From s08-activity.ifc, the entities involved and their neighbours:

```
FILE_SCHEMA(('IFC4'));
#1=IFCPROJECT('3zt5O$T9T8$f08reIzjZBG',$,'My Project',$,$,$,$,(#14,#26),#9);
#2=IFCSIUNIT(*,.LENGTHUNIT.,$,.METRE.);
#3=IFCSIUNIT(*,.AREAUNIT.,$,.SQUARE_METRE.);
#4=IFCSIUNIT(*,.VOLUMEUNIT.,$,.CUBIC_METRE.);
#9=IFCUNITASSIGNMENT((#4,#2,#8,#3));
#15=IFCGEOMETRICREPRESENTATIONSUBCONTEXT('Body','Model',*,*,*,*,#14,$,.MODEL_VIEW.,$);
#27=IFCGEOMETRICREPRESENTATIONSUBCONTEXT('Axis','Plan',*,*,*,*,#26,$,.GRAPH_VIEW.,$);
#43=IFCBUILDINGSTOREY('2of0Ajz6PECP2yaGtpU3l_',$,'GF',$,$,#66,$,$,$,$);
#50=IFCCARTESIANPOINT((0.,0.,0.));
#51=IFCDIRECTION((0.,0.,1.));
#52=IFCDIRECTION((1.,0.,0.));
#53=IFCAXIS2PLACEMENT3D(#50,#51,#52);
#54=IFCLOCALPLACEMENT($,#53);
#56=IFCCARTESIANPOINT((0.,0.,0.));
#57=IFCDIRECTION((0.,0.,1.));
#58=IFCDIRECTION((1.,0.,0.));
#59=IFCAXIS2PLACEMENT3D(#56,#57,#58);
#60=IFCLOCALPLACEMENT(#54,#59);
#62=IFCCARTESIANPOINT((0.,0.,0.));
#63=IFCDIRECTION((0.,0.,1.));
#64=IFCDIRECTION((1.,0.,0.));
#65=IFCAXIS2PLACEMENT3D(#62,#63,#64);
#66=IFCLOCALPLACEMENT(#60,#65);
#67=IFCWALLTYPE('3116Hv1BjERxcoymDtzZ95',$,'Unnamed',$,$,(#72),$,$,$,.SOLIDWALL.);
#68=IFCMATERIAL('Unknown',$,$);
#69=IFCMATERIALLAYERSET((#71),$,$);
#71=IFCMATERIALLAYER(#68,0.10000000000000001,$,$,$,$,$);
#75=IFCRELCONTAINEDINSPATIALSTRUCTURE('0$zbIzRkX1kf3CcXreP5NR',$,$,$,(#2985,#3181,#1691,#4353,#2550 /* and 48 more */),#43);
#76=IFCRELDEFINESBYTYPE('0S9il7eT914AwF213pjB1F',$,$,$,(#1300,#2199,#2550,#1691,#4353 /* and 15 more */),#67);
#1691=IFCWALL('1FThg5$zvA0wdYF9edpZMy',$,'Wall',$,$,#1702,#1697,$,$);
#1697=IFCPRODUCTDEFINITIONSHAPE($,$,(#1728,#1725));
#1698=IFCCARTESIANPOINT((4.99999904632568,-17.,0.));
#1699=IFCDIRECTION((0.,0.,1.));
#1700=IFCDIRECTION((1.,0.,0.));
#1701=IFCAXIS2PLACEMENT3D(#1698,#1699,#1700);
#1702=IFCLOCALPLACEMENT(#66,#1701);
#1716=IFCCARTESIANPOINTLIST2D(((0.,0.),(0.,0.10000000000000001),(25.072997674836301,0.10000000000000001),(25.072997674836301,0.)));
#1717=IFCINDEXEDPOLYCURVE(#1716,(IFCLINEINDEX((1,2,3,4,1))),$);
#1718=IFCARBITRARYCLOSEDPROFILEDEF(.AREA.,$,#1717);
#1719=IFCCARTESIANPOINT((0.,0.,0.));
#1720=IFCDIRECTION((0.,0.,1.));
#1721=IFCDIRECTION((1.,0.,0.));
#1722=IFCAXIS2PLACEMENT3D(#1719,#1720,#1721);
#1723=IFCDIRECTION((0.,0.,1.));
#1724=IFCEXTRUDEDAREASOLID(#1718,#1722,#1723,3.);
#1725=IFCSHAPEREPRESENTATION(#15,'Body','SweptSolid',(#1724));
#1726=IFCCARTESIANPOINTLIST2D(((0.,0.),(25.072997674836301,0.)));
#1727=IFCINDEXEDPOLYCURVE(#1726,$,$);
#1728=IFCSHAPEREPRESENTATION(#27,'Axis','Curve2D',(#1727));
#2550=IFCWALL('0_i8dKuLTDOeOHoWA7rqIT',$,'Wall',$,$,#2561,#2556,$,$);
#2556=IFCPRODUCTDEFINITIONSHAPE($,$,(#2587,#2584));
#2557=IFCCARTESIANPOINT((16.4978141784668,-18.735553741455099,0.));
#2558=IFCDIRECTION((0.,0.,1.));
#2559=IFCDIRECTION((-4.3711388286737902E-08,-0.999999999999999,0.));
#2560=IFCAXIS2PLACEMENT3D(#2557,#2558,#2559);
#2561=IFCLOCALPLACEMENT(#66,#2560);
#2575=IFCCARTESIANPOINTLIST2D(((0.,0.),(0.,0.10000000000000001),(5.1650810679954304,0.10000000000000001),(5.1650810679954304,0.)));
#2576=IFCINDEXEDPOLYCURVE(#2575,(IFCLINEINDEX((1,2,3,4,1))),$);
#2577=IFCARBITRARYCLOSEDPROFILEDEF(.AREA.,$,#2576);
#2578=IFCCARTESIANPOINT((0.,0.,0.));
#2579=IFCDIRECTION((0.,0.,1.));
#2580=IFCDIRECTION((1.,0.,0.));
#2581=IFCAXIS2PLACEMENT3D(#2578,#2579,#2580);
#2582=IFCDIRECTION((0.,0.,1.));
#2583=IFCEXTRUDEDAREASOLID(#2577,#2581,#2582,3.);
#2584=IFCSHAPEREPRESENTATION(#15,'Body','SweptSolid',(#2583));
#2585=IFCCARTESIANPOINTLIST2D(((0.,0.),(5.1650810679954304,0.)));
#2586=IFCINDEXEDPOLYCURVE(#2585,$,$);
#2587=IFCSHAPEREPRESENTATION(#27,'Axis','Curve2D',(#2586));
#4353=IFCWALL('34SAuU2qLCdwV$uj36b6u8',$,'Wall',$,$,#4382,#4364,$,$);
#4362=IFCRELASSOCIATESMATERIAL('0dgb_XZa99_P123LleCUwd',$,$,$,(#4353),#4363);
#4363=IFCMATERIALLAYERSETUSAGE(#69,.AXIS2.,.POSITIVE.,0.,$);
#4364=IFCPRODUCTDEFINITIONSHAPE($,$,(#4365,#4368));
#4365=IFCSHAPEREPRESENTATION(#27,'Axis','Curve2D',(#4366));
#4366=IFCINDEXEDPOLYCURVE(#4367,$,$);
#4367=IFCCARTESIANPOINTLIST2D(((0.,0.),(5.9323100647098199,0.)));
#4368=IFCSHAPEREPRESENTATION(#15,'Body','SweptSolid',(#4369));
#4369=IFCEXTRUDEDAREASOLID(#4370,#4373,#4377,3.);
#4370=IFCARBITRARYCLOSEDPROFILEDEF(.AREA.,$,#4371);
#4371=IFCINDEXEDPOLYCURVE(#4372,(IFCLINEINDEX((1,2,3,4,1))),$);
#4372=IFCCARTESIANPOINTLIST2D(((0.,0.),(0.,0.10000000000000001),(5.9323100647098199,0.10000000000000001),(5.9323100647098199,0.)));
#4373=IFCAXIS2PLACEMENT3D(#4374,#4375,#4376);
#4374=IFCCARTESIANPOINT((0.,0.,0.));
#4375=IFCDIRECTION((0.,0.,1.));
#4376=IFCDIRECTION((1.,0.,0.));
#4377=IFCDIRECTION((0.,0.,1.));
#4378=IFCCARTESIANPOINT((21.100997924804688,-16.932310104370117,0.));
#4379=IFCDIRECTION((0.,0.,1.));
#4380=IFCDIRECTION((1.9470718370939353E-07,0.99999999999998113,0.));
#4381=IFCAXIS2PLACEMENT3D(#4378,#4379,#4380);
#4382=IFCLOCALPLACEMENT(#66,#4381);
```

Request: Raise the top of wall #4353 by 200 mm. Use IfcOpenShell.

```python
import ifcopenshell
import ifcopenshell.geom
import ifcopenshell.util.representation
import ifcopenshell.util.shape
import ifcopenshell.util.unit

model = ifcopenshell.open("s08-activity.ifc")
unit_scale = ifcopenshell.util.unit.calculate_unit_scale(model)
settings = ifcopenshell.geom.settings()


def volume(element):
    """Net volume in cubic metres, openings subtracted."""
    shape = ifcopenshell.geom.create_shape(settings, element)
    return ifcopenshell.util.shape.get_volume(shape.geometry)


wall = model.by_guid("34SAuU2qLCdwV$uj36b6u8")
before = volume(wall)

body = ifcopenshell.util.representation.get_representation(wall, "Model", "Body")
solid = body.Items[0]
old_height = solid.Depth
solid.Depth += 0.2 / unit_scale
after = volume(wall)

print(f"height {old_height:g} -> {solid.Depth:g}, volume {before:.3f} -> {after:.3f} m3")

model.write("s08-activity-out.ifc")
```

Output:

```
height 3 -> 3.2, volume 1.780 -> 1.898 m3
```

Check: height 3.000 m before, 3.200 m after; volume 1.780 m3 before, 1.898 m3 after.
